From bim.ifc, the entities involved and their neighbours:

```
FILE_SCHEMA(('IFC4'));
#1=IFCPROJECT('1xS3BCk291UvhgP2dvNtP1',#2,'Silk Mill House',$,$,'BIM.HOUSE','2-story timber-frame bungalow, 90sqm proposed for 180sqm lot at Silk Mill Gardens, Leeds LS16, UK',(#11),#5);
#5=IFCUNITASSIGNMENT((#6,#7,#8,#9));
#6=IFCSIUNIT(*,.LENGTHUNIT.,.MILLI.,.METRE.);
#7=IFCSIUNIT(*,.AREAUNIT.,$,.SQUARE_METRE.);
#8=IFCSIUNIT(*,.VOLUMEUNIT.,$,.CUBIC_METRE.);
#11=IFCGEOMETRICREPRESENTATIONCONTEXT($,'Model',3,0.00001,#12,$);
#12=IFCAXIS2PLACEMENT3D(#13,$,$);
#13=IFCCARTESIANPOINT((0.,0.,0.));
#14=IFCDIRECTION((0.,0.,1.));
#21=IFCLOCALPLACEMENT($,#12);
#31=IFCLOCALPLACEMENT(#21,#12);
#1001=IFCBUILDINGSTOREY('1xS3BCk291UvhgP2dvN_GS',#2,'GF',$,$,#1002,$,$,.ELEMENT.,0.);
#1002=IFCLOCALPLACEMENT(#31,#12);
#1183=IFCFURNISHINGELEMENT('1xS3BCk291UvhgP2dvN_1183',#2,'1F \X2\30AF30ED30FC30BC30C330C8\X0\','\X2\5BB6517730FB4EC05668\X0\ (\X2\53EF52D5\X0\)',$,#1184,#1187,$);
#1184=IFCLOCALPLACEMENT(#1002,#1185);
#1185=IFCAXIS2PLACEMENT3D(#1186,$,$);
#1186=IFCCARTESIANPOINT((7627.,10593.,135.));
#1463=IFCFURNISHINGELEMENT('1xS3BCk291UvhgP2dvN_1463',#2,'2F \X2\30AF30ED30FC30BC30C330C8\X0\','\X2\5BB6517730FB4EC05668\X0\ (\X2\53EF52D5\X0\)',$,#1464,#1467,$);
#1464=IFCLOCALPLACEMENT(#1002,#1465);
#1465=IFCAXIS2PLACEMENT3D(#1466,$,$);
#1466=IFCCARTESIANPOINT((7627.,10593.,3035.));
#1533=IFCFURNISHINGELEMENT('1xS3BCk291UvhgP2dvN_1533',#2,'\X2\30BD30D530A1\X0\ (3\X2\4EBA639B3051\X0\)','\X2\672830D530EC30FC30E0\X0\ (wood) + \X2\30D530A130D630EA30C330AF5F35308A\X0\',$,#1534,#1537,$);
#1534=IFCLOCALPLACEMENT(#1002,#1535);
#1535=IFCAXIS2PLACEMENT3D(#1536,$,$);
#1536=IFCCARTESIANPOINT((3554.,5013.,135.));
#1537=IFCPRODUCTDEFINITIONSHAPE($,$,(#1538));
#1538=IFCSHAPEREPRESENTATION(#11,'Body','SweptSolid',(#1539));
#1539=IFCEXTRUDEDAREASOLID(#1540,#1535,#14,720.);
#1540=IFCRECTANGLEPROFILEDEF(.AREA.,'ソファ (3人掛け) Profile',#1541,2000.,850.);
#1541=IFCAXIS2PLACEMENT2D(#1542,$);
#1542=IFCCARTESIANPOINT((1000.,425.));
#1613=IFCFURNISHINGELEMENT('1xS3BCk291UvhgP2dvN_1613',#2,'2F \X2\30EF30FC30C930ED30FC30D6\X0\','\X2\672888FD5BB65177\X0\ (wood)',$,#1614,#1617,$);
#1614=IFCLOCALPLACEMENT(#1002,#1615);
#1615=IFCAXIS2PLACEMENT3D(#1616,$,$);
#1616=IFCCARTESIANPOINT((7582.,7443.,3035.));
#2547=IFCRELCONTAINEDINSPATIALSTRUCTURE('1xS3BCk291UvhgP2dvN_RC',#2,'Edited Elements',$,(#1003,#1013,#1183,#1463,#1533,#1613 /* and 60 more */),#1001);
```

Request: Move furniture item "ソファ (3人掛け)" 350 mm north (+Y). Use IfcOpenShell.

```python
import ifcopenshell
import ifcopenshell.api.geometry
import ifcopenshell.util.placement
import ifcopenshell.util.unit

model = ifcopenshell.open("bim.ifc")
unit_scale = ifcopenshell.util.unit.calculate_unit_scale(model)

item = model.by_guid("1xS3BCk291UvhgP2dvN_1533")
matrix = ifcopenshell.util.placement.get_local_placement(item.ObjectPlacement)
matrix[1, 3] += 0.35 / unit_scale
ifcopenshell.api.geometry.edit_object_placement(model, product=item, matrix=matrix, is_si=False)

print(ifcopenshell.util.placement.get_local_placement(item.ObjectPlacement).round(3) + 0.0)

model.write("bim_edited.ifc")
```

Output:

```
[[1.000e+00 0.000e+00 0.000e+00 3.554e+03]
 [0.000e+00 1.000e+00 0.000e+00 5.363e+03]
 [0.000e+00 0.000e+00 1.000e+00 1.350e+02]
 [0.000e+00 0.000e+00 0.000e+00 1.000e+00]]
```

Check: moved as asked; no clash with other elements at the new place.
